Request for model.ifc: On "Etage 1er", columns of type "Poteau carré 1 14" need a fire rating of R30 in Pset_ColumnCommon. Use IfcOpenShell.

First a look at what the model holds.

```python
import ifcopenshell
import ifcopenshell.util.element

model = ifcopenshell.open("model.ifc")
print(model.schema)
storey = next(s for s in model.by_type("IfcBuildingStorey") if s.Name == "Etage 1er")
columns = [e for e in ifcopenshell.util.element.get_decomposition(storey) if e.is_a("IfcColumn")]
seen = {}
for e in columns:
    element_type = ifcopenshell.util.element.get_type(e)
    key = (element_type.Name if element_type != e and element_type else None, ifcopenshell.util.element.get_pset(e, "Pset_ColumnCommon", "FireRating"))
    seen[key] = seen.get(key, 0) + 1
for (name, value), count in sorted(seen.items(), key=str):
    print(count, "x", name, "|", value)
```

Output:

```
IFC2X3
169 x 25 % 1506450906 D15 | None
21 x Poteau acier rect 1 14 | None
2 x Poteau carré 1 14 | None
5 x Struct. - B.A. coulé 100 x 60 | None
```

```python
import ifcopenshell
import ifcopenshell.api.pset
import ifcopenshell.util.element

model = ifcopenshell.open("model.ifc")

storey = next(s for s in model.by_type("IfcBuildingStorey") if s.Name == "Etage 1er")
columns = [e for e in ifcopenshell.util.element.get_decomposition(storey) if e.is_a("IfcColumn")]

count = 0
for e in columns:
    element_type = ifcopenshell.util.element.get_type(e)
    if element_type in (None, e) or element_type.Name != "Poteau carré 1 14":
        continue
    # add_pset returns the element's existing set when there is one.
    pset = ifcopenshell.api.pset.add_pset(model, product=e, name="Pset_ColumnCommon")
    ifcopenshell.api.pset.edit_pset(model, pset=pset, properties={"FireRating": "R30"})
    count += 1

print(count, "columns updated")

model.write("model_edited.ifc")
```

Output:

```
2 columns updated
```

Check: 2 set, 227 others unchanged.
